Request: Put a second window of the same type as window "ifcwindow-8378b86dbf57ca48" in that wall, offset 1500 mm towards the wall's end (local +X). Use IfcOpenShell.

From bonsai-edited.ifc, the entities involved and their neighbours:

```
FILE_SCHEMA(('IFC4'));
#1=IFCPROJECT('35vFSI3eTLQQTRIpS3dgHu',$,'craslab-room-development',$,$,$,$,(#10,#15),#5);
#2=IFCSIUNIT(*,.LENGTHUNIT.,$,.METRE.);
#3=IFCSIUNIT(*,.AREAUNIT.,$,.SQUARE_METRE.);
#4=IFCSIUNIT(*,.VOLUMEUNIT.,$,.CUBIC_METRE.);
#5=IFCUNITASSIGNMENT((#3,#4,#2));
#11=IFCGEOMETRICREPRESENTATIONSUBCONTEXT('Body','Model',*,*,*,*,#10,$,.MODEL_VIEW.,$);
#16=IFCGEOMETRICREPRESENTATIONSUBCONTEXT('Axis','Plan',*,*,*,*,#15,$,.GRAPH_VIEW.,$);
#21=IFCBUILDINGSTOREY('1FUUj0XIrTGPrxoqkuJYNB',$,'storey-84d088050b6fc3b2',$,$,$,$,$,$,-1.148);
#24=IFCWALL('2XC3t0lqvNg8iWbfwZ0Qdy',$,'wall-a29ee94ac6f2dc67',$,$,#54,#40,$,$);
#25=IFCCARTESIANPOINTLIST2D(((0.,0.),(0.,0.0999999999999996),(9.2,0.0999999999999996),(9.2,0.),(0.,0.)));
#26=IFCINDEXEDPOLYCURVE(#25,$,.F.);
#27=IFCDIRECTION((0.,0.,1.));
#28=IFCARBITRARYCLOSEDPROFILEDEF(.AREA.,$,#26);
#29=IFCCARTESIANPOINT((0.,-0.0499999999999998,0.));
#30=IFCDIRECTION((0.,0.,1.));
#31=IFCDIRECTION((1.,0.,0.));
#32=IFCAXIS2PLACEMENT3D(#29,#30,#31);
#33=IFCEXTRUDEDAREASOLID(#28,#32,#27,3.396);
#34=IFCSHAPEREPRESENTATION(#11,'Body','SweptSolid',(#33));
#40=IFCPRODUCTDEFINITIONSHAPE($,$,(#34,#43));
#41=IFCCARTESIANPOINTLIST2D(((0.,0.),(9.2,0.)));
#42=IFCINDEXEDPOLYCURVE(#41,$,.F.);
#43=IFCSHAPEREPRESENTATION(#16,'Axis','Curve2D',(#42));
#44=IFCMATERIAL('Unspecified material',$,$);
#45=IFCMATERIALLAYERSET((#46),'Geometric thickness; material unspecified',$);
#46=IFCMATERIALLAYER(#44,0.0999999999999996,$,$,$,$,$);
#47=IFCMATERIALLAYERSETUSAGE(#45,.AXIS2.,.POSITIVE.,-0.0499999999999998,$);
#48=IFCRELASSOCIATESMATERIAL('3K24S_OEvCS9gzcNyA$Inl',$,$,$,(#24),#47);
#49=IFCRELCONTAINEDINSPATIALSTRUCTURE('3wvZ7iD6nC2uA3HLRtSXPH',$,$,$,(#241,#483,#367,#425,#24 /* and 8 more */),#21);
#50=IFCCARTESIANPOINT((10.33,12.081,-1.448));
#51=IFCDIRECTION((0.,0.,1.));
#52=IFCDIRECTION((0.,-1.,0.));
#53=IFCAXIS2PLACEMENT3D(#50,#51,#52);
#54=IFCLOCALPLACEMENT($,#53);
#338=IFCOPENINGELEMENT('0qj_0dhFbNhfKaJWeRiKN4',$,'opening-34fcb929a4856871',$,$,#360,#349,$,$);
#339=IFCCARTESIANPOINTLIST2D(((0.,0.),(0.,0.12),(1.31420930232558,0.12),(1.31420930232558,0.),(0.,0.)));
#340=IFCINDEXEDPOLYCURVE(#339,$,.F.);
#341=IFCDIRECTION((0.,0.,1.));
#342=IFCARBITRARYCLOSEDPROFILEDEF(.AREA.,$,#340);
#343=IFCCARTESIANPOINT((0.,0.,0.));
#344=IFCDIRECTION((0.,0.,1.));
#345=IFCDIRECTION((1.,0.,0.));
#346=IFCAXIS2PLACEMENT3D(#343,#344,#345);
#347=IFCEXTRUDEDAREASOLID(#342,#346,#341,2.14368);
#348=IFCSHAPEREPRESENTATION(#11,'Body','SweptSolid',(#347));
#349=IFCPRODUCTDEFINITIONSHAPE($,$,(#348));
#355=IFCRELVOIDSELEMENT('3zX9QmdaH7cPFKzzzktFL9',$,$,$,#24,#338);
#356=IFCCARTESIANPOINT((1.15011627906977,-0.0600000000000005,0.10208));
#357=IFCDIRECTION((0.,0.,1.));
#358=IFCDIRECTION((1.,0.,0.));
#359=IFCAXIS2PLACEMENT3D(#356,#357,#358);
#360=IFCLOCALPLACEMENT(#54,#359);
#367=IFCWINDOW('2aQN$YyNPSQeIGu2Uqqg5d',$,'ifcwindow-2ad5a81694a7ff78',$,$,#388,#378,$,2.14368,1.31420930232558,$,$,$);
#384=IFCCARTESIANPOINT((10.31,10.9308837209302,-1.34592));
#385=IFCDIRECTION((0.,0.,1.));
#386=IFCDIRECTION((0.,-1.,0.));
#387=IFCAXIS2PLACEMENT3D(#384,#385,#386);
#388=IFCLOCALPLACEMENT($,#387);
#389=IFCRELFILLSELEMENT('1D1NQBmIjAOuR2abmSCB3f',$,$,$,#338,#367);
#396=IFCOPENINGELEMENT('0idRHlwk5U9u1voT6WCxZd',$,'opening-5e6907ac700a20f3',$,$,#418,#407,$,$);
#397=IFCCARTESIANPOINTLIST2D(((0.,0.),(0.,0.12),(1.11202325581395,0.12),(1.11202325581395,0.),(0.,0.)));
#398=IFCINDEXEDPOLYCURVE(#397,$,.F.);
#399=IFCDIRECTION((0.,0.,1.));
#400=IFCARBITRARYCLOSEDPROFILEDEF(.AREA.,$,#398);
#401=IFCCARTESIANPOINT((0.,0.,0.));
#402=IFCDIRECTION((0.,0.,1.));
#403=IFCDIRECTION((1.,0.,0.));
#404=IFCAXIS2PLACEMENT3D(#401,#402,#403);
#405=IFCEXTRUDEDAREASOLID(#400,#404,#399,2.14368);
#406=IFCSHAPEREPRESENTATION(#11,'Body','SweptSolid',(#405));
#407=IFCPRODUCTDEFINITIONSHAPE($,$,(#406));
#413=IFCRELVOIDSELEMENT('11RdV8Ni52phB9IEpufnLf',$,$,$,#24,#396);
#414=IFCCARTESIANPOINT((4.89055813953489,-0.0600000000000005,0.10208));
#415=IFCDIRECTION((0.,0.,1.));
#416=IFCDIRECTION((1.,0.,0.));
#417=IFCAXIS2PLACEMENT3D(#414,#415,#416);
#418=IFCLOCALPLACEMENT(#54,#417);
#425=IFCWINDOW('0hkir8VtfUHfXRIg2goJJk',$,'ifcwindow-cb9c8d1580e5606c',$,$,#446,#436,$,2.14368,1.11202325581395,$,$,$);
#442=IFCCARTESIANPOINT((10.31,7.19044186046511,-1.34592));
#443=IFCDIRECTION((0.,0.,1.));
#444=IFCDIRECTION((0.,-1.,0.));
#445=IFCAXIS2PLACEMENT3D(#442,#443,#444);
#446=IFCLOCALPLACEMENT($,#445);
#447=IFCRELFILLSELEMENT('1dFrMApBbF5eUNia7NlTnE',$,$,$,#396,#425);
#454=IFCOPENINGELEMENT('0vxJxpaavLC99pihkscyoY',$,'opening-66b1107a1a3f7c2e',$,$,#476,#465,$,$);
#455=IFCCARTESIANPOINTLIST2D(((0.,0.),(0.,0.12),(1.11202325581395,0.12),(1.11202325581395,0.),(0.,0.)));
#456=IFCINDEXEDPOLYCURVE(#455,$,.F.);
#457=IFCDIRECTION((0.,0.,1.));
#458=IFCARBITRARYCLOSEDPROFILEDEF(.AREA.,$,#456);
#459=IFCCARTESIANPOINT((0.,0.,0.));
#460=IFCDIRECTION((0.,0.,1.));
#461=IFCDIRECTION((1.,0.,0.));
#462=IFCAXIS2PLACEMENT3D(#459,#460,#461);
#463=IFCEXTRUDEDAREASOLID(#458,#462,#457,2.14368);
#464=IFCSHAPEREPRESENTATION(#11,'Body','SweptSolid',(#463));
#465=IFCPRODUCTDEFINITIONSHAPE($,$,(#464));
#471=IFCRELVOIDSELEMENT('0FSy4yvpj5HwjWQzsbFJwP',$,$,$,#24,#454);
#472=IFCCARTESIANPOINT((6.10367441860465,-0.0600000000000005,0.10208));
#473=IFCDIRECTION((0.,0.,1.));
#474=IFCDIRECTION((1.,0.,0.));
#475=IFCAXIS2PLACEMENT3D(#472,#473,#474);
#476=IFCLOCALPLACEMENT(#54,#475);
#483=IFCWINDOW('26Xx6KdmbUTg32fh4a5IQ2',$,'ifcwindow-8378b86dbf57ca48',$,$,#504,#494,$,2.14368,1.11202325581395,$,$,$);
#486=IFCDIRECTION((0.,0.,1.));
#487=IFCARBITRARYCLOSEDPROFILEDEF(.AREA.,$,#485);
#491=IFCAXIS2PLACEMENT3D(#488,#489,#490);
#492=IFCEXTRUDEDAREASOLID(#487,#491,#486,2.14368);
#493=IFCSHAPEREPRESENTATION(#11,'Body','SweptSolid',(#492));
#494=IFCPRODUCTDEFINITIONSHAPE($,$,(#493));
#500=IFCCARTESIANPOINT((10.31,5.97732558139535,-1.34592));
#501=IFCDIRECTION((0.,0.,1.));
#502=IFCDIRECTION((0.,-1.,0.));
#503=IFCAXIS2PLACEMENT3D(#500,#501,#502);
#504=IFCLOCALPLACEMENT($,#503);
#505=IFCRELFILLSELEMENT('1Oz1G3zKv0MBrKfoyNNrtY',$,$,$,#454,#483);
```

```python
import ifcopenshell
import ifcopenshell.api.feature
import ifcopenshell.api.geometry
import ifcopenshell.api.root
import ifcopenshell.geom
import ifcopenshell.util.element
import ifcopenshell.util.placement
import ifcopenshell.util.shape

model = ifcopenshell.open("bonsai-edited.ifc")
settings = ifcopenshell.geom.settings()


def volume(element):
    """Net volume in cubic metres, openings subtracted."""
    shape = ifcopenshell.geom.create_shape(settings, element)
    return ifcopenshell.util.shape.get_volume(shape.geometry)


window = model.by_id(483)
opening = window.FillsVoids[0].RelatingOpeningElement
wall = opening.VoidsElements[0].RelatingBuildingElement
before = volume(wall)
shift = ifcopenshell.util.placement.get_local_placement(wall.ObjectPlacement)[:3, 0] * 1.5

# copy_class copies the void relationship, type, container and properties, but no geometry.
new_opening = ifcopenshell.api.root.copy_class(model, product=opening)
new_opening.Representation = ifcopenshell.util.element.copy_deep(
    model, opening.Representation, exclude=["IfcGeometricRepresentationContext", "IfcRepresentationMap"]
)
new_window = ifcopenshell.api.root.copy_class(model, product=window)
new_window.Representation = ifcopenshell.util.element.copy_deep(
    model, window.Representation, exclude=["IfcGeometricRepresentationContext", "IfcRepresentationMap"]
)
ifcopenshell.api.feature.add_filling(model, opening=new_opening, element=new_window)

for old, new in ((opening, new_opening), (window, new_window)):
    matrix = ifcopenshell.util.placement.get_local_placement(old.ObjectPlacement)
    matrix[:3, 3] += shift
    ifcopenshell.api.geometry.edit_object_placement(model, product=new, matrix=matrix, is_si=False)

after = volume(wall)

print(f"wall volume {before:.3f} -> {after:.3f} m3")

model.write("bonsai-edited-out.ifc")
```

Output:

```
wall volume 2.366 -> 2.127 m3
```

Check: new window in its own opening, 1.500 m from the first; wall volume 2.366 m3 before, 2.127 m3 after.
